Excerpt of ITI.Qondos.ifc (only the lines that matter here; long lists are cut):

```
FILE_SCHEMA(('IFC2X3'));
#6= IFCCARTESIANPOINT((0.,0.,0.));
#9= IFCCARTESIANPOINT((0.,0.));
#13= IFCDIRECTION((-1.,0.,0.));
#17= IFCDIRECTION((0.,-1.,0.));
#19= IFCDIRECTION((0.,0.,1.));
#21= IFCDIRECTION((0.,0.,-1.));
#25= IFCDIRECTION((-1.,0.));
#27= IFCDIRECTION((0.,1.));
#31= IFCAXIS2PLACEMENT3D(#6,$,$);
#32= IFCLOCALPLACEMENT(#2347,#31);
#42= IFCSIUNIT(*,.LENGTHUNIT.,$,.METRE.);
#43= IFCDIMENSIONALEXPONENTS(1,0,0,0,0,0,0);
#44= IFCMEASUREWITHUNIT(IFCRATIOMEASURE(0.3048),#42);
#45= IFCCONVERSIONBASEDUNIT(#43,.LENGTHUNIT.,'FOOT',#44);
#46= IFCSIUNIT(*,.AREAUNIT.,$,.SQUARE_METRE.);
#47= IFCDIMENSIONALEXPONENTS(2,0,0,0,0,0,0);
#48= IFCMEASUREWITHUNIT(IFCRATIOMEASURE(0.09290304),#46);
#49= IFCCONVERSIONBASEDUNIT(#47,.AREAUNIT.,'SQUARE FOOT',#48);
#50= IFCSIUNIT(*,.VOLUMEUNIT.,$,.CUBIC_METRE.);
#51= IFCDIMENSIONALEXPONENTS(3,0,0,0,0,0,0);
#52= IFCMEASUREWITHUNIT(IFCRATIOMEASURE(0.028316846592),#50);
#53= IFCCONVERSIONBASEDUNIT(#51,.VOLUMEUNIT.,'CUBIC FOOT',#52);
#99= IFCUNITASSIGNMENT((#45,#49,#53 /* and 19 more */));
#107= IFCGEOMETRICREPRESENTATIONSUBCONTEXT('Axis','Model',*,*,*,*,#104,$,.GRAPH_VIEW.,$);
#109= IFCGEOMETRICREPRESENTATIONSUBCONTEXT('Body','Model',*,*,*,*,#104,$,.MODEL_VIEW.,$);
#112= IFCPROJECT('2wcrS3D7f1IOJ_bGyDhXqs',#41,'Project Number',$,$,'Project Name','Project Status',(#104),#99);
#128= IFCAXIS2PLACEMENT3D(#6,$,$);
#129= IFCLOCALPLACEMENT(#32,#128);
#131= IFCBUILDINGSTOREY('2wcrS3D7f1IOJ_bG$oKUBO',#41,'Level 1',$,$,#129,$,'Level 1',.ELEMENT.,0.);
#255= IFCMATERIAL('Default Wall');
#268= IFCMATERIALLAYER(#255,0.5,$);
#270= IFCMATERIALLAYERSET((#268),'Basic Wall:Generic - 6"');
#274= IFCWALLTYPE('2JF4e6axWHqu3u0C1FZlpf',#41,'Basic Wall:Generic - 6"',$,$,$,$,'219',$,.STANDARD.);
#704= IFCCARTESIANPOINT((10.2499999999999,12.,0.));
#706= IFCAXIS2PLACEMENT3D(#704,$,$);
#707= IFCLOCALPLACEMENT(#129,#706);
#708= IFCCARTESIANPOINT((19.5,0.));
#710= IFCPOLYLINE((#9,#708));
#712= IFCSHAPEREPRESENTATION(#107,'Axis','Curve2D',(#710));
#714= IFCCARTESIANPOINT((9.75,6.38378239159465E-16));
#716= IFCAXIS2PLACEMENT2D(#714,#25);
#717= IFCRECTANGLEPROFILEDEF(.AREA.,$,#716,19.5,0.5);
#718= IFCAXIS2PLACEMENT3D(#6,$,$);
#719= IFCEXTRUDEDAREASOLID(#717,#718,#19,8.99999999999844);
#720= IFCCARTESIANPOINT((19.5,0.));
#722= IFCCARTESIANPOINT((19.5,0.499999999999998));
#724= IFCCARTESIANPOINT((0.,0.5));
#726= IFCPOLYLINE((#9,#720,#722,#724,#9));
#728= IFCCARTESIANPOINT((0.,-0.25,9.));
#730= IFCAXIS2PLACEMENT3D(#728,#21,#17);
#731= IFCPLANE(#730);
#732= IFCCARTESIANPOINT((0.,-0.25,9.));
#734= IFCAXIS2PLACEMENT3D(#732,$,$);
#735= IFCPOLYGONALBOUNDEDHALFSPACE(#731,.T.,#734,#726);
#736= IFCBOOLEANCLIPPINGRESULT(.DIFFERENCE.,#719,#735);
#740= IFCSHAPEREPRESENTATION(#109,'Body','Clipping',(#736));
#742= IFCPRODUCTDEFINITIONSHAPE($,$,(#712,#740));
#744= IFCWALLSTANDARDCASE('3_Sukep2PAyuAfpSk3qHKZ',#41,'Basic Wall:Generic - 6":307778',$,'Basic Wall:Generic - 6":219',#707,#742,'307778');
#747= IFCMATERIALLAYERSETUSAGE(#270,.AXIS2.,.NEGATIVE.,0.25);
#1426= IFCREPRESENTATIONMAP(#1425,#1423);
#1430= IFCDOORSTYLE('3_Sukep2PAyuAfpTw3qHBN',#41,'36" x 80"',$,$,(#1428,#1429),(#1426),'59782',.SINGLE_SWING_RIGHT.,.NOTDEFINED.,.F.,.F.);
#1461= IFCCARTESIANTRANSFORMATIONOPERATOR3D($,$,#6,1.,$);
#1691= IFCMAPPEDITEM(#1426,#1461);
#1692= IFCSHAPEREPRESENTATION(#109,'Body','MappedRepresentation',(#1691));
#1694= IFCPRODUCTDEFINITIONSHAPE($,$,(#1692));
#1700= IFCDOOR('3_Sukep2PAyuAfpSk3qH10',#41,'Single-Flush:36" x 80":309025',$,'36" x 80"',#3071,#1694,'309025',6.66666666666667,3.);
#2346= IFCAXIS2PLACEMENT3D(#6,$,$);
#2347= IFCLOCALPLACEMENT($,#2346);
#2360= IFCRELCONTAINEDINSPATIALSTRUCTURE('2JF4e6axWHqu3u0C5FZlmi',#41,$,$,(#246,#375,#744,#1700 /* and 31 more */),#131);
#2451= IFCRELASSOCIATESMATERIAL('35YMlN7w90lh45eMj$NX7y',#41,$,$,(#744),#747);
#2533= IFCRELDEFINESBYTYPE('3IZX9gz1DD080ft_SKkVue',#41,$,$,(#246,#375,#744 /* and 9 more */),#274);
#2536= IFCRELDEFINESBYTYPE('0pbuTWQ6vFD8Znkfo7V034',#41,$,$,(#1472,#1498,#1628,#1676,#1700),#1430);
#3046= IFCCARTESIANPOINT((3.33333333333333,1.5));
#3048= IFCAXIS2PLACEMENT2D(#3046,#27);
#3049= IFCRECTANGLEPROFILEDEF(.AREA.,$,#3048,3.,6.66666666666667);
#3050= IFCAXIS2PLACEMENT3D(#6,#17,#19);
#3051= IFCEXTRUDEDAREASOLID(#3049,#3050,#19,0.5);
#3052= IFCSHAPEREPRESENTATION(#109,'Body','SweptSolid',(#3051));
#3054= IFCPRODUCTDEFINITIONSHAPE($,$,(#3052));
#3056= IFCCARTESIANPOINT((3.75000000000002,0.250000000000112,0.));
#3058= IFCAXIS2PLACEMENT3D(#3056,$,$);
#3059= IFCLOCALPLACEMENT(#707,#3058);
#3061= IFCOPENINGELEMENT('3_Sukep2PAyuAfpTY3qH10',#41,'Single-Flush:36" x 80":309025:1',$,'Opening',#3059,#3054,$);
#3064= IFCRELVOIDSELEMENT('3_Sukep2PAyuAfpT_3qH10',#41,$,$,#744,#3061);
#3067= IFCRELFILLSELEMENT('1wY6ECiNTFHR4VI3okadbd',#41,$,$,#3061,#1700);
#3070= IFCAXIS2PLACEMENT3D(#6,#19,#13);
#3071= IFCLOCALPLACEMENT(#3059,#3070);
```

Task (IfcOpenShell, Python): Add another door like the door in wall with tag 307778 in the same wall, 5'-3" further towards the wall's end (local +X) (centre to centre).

```python
import ifcopenshell
import ifcopenshell.api.feature
import ifcopenshell.api.geometry
import ifcopenshell.api.root
import ifcopenshell.geom
import ifcopenshell.util.element
import ifcopenshell.util.placement
import ifcopenshell.util.shape
import ifcopenshell.util.unit

model = ifcopenshell.open("ITI.Qondos.ifc")
unit_scale = ifcopenshell.util.unit.calculate_unit_scale(model)
settings = ifcopenshell.geom.settings()


def volume(element):
    """Net volume in cubic metres, openings subtracted."""
    shape = ifcopenshell.geom.create_shape(settings, element)
    return ifcopenshell.util.shape.get_volume(shape.geometry)


def reuse_history(source, copy):
    """copy_class also copies each property set's owner history, people and application; keep the originals."""
    for rel in copy.IsDefinedBy:
        if rel.is_a("IfcRelDefinesByProperties") and (history := rel.RelatingPropertyDefinition.OwnerHistory):
            rel.RelatingPropertyDefinition.OwnerHistory = source.OwnerHistory
            ifcopenshell.util.element.remove_deep2(model, history)


door = model.by_id(1700)
opening = door.FillsVoids[0].RelatingOpeningElement
wall = opening.VoidsElements[0].RelatingBuildingElement
before = volume(wall)
shift = ifcopenshell.util.placement.get_local_placement(wall.ObjectPlacement)[:3, 0] * 63 * 0.0254 / unit_scale

# copy_class copies the void relationship, type, container and properties, but no geometry.
new_opening = ifcopenshell.api.root.copy_class(model, product=opening)
new_opening.Representation = ifcopenshell.util.element.copy_deep(
    model, opening.Representation, exclude=["IfcGeometricRepresentationContext", "IfcRepresentationMap"]
)
new_opening.Name = 'Single-Flush:36" x 80"'
new_door = ifcopenshell.api.root.copy_class(model, product=door)
new_door.Representation = ifcopenshell.util.element.copy_deep(
    model, door.Representation, exclude=["IfcGeometricRepresentationContext", "IfcRepresentationMap"]
)
new_door.Name = 'Single-Flush:36" x 80"'
new_door.Tag = None
reuse_history(door, new_door)
fills = ifcopenshell.api.feature.add_filling(model, opening=new_opening, element=new_door)
fills.OwnerHistory = new_door.OwnerHistory  # required in IFC2X3

for old, new in ((opening, new_opening), (door, new_door)):
    matrix = ifcopenshell.util.placement.get_local_placement(old.ObjectPlacement)
    matrix[:3, 3] += shift
    ifcopenshell.api.geometry.edit_object_placement(model, product=new, matrix=matrix, is_si=False)

after = volume(wall)

print(f"wall volume {before:.3f} -> {after:.3f} m3")

model.write("ITI.Qondos_updated.ifc")
```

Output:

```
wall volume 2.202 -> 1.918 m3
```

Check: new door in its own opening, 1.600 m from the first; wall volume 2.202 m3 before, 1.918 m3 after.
